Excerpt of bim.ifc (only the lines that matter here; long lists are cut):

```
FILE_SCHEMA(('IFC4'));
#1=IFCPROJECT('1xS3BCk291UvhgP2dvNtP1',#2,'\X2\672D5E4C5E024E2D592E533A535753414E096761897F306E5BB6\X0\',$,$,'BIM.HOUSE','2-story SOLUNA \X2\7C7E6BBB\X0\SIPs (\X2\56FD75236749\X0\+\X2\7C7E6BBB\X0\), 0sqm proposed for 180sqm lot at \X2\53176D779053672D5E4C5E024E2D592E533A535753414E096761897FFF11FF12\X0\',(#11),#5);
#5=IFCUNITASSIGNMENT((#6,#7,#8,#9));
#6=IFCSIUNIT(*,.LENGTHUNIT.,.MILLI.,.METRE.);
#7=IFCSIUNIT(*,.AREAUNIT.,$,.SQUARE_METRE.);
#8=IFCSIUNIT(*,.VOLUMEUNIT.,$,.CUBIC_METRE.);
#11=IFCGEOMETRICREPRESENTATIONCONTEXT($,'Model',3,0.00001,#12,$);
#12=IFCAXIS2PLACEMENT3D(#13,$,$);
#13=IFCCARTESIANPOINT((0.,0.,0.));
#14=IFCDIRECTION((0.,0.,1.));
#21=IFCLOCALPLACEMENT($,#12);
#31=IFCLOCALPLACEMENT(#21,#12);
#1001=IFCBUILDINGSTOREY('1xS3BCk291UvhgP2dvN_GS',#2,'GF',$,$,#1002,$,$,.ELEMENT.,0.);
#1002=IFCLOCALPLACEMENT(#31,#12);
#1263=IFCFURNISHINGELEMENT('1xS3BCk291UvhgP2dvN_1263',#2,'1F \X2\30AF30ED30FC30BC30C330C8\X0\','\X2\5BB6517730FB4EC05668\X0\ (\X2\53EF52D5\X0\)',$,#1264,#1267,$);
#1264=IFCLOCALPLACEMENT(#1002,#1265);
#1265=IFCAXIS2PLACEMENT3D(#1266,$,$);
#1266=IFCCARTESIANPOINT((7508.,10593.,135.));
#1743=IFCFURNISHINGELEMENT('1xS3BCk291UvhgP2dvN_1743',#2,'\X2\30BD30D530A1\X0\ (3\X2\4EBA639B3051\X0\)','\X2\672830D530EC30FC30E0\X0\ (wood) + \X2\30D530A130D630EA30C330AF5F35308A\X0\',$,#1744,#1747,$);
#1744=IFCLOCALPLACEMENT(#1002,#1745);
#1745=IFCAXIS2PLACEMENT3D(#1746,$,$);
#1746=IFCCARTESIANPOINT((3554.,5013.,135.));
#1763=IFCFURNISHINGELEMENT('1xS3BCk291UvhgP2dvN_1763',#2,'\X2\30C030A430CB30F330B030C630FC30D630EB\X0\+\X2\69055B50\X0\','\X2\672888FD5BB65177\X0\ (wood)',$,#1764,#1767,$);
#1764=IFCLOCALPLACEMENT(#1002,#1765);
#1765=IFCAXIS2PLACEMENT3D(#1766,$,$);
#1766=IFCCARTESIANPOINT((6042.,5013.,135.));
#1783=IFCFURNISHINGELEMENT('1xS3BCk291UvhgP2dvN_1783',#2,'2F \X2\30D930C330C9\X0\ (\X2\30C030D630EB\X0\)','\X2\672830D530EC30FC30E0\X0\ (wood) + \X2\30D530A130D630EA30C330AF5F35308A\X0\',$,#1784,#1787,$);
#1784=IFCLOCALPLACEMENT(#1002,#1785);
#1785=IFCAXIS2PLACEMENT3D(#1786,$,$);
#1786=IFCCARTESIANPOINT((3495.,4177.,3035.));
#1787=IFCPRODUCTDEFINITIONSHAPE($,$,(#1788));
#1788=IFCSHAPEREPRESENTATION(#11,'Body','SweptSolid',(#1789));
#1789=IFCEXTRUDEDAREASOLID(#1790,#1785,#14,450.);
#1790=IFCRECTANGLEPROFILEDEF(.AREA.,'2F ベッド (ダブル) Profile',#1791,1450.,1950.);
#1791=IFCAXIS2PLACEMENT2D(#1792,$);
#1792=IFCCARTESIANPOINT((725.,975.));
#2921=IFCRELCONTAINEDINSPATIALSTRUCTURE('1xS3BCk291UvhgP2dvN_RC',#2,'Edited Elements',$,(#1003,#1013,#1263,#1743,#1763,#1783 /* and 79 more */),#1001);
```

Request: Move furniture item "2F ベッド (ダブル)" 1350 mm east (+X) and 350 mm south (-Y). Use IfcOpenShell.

```python
import ifcopenshell
import ifcopenshell.api.geometry
import ifcopenshell.util.placement
import ifcopenshell.util.unit

model = ifcopenshell.open("bim.ifc")
unit_scale = ifcopenshell.util.unit.calculate_unit_scale(model)

item = model.by_guid("1xS3BCk291UvhgP2dvN_1783")
matrix = ifcopenshell.util.placement.get_local_placement(item.ObjectPlacement)
matrix[0, 3] += 1.35 / unit_scale
matrix[1, 3] -= 0.35 / unit_scale
ifcopenshell.api.geometry.edit_object_placement(model, product=item, matrix=matrix, is_si=False)

print(ifcopenshell.util.placement.get_local_placement(item.ObjectPlacement).round(3) + 0.0)

model.write("bim_rev.ifc")
```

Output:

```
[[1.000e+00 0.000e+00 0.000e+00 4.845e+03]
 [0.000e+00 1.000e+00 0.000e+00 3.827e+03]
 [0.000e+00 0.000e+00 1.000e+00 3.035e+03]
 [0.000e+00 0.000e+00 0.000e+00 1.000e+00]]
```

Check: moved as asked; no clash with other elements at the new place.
